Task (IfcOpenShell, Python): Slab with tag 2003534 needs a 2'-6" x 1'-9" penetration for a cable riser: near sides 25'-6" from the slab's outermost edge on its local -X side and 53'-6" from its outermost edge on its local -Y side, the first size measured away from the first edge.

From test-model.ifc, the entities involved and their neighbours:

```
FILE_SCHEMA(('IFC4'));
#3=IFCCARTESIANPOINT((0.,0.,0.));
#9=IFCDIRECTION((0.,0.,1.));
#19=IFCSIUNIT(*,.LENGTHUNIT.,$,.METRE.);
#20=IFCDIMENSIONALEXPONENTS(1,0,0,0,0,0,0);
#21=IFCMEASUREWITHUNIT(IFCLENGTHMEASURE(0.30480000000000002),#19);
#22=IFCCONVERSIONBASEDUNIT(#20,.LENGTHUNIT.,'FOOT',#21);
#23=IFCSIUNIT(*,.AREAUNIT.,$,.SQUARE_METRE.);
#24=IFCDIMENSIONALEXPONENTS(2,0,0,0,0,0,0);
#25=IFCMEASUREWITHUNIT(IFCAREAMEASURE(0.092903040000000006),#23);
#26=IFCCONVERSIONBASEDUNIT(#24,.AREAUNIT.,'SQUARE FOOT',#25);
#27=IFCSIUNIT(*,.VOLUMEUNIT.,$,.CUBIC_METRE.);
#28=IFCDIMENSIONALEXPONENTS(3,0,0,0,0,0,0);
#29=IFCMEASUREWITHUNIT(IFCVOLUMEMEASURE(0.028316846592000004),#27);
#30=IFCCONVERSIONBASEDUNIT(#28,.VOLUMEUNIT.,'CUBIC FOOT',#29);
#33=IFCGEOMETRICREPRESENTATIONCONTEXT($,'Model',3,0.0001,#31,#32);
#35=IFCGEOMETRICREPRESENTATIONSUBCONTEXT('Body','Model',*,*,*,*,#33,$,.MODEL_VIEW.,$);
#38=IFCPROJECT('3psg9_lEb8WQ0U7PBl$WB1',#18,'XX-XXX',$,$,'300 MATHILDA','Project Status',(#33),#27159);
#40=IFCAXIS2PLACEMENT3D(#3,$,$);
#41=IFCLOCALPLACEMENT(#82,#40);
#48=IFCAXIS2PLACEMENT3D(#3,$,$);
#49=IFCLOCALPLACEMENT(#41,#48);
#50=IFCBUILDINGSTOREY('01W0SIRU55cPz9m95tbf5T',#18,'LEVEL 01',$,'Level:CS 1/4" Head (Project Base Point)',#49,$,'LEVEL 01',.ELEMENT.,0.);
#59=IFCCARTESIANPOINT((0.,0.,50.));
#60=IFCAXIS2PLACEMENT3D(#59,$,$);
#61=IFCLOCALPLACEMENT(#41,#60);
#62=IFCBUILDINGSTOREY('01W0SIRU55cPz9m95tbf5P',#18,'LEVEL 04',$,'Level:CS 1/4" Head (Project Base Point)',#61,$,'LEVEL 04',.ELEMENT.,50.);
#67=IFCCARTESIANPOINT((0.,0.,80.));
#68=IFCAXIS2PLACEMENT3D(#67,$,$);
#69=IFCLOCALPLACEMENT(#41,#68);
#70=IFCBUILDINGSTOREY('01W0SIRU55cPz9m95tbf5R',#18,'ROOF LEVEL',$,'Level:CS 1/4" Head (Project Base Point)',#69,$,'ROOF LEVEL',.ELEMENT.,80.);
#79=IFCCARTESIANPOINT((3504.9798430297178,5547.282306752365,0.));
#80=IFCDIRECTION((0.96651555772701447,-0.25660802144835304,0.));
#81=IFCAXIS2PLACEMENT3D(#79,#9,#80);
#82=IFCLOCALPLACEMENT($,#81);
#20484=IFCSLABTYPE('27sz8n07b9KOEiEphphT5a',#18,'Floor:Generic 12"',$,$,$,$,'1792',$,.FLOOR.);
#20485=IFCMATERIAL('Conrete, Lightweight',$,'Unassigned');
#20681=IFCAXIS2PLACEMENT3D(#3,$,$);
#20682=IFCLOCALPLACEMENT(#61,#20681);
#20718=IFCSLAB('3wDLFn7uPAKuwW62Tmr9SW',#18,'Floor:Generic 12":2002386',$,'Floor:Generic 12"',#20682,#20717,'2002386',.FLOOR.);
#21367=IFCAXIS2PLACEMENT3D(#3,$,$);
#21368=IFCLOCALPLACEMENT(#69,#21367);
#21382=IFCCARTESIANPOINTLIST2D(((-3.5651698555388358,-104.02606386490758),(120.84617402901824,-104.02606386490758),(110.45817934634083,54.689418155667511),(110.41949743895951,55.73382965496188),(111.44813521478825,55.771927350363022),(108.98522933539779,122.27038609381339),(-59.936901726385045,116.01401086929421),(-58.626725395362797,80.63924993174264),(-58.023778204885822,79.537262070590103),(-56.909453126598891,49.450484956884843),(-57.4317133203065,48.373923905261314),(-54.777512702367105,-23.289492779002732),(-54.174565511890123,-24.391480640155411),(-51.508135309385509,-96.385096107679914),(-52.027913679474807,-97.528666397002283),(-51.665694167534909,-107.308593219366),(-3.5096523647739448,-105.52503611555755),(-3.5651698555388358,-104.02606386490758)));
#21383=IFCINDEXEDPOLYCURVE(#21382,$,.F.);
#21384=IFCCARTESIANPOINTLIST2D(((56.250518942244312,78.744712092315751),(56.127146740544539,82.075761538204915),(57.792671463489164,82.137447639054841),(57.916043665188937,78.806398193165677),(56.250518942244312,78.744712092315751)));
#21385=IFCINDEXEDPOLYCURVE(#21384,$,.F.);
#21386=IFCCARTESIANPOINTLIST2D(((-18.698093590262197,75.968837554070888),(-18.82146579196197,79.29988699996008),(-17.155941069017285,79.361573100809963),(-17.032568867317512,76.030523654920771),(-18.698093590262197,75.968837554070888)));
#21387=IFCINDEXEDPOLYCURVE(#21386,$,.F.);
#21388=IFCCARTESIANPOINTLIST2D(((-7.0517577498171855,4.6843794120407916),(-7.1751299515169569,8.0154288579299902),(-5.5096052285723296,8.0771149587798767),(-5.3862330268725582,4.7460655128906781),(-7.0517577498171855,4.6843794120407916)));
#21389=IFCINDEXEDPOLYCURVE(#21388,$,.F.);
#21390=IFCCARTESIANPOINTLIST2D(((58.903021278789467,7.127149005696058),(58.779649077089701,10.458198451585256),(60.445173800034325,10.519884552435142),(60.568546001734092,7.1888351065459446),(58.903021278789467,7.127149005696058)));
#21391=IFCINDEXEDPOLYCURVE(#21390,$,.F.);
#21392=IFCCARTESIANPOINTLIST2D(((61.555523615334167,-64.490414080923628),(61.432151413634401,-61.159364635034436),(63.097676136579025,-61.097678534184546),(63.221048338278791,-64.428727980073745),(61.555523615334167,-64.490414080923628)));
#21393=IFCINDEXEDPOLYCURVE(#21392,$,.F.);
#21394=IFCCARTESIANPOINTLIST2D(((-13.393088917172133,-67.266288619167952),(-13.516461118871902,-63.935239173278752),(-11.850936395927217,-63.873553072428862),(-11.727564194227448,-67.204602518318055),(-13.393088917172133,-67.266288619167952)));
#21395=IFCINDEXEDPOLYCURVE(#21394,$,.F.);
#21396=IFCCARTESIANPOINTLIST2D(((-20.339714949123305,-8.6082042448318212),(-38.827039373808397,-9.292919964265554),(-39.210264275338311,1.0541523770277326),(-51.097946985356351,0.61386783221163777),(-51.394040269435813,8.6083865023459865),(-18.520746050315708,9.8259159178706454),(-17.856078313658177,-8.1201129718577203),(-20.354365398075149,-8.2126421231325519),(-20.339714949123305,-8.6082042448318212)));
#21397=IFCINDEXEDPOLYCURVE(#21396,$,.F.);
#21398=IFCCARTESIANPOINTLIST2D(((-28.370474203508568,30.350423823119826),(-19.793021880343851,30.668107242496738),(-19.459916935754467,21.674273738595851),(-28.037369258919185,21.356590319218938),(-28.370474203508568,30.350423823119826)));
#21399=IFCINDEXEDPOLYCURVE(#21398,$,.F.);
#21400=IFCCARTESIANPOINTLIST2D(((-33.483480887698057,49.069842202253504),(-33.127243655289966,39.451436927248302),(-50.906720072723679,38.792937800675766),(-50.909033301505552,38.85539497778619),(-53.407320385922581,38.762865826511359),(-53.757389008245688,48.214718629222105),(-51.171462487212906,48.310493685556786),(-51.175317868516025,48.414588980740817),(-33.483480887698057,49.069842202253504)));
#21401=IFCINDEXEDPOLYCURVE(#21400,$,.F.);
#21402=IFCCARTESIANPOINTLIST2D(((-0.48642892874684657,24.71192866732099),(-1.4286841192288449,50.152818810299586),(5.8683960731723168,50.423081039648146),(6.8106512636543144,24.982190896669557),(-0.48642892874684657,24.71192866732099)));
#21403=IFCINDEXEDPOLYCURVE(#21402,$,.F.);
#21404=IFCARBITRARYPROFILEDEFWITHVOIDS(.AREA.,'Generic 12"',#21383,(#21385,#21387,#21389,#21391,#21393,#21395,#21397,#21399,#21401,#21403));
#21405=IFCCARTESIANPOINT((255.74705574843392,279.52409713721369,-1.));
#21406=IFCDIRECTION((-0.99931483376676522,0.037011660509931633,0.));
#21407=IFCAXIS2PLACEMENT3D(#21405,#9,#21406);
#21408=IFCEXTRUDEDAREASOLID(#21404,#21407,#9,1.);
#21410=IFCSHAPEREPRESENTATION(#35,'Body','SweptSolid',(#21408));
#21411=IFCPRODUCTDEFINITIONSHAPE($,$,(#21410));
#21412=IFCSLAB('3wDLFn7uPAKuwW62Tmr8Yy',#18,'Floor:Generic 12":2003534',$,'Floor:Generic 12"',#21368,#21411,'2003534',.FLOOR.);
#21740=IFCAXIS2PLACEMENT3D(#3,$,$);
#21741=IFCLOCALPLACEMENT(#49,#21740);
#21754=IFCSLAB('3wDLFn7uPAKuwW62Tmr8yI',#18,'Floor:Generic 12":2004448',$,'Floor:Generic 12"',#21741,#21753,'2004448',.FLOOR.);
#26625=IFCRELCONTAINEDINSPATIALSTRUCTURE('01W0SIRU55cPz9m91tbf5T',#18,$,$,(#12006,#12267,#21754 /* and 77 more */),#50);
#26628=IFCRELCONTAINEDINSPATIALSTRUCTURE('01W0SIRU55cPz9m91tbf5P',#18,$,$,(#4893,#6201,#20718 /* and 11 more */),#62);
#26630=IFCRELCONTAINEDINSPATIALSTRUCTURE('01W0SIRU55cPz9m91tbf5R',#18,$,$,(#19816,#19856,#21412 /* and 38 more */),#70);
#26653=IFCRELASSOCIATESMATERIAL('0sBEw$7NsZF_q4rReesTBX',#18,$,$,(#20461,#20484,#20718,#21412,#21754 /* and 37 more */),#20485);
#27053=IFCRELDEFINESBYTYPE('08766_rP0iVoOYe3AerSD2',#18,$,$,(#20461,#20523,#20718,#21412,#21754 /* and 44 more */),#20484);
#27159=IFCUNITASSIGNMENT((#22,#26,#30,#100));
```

```python
import numpy as np
import ifcopenshell
import ifcopenshell.api.feature
import ifcopenshell.api.geometry
import ifcopenshell.api.root
import ifcopenshell.geom
import ifcopenshell.util.placement
import ifcopenshell.util.representation
import ifcopenshell.util.shape
import ifcopenshell.util.unit

model = ifcopenshell.open("test-model.ifc")
unit_scale = ifcopenshell.util.unit.calculate_unit_scale(model)
settings = ifcopenshell.geom.settings()


def volume(element):
    """Net volume in cubic metres, openings subtracted."""
    shape = ifcopenshell.geom.create_shape(settings, element)
    return ifcopenshell.util.shape.get_volume(shape.geometry)


slab = model.by_id(21412)
before = volume(slab)

# Extent in the slab's own axes, in metres. The edges named are its -X and -Y sides.
slab_shape = ifcopenshell.geom.create_shape(settings, slab)
vertices = ifcopenshell.util.shape.get_vertices(slab_shape.geometry)
x_min, y_min, bottom = vertices.min(axis=0)
top = vertices[:, 2].max()

opening = ifcopenshell.api.root.create_entity(model, ifc_class="IfcOpeningElement", name="Cable riser opening", predefined_type="OPENING")
context = ifcopenshell.util.representation.get_context(model, "Model", "Body", "MODEL_VIEW")
width, depth = 0.762, 0.5334
outline = [(0.0, 0.0), (width, 0.0), (width, depth), (0.0, depth), (0.0, 0.0)]
# Overshoot both faces by 50 mm so the cut is clean.
shape = ifcopenshell.api.geometry.add_slab_representation(
    model, context=context, depth=top - bottom + 0.1, polyline=outline
)
ifcopenshell.api.geometry.assign_representation(model, product=opening, representation=shape)

matrix = ifcopenshell.util.placement.get_local_placement(slab.ObjectPlacement)
matrix[:, 3] = matrix @ np.append(np.array([x_min + 7.7724, y_min + 16.3068, bottom - 0.05]) / unit_scale, 1.0)
ifcopenshell.api.geometry.edit_object_placement(model, product=opening, matrix=matrix, is_si=False)
ifcopenshell.api.feature.add_feature(model, feature=opening, element=slab)

after = volume(slab)

print(f"slab volume {before:.3f} -> {after:.3f} m3")

model.write("test-model-out.ifc")
```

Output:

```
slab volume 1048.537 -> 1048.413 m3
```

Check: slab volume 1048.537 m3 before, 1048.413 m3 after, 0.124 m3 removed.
